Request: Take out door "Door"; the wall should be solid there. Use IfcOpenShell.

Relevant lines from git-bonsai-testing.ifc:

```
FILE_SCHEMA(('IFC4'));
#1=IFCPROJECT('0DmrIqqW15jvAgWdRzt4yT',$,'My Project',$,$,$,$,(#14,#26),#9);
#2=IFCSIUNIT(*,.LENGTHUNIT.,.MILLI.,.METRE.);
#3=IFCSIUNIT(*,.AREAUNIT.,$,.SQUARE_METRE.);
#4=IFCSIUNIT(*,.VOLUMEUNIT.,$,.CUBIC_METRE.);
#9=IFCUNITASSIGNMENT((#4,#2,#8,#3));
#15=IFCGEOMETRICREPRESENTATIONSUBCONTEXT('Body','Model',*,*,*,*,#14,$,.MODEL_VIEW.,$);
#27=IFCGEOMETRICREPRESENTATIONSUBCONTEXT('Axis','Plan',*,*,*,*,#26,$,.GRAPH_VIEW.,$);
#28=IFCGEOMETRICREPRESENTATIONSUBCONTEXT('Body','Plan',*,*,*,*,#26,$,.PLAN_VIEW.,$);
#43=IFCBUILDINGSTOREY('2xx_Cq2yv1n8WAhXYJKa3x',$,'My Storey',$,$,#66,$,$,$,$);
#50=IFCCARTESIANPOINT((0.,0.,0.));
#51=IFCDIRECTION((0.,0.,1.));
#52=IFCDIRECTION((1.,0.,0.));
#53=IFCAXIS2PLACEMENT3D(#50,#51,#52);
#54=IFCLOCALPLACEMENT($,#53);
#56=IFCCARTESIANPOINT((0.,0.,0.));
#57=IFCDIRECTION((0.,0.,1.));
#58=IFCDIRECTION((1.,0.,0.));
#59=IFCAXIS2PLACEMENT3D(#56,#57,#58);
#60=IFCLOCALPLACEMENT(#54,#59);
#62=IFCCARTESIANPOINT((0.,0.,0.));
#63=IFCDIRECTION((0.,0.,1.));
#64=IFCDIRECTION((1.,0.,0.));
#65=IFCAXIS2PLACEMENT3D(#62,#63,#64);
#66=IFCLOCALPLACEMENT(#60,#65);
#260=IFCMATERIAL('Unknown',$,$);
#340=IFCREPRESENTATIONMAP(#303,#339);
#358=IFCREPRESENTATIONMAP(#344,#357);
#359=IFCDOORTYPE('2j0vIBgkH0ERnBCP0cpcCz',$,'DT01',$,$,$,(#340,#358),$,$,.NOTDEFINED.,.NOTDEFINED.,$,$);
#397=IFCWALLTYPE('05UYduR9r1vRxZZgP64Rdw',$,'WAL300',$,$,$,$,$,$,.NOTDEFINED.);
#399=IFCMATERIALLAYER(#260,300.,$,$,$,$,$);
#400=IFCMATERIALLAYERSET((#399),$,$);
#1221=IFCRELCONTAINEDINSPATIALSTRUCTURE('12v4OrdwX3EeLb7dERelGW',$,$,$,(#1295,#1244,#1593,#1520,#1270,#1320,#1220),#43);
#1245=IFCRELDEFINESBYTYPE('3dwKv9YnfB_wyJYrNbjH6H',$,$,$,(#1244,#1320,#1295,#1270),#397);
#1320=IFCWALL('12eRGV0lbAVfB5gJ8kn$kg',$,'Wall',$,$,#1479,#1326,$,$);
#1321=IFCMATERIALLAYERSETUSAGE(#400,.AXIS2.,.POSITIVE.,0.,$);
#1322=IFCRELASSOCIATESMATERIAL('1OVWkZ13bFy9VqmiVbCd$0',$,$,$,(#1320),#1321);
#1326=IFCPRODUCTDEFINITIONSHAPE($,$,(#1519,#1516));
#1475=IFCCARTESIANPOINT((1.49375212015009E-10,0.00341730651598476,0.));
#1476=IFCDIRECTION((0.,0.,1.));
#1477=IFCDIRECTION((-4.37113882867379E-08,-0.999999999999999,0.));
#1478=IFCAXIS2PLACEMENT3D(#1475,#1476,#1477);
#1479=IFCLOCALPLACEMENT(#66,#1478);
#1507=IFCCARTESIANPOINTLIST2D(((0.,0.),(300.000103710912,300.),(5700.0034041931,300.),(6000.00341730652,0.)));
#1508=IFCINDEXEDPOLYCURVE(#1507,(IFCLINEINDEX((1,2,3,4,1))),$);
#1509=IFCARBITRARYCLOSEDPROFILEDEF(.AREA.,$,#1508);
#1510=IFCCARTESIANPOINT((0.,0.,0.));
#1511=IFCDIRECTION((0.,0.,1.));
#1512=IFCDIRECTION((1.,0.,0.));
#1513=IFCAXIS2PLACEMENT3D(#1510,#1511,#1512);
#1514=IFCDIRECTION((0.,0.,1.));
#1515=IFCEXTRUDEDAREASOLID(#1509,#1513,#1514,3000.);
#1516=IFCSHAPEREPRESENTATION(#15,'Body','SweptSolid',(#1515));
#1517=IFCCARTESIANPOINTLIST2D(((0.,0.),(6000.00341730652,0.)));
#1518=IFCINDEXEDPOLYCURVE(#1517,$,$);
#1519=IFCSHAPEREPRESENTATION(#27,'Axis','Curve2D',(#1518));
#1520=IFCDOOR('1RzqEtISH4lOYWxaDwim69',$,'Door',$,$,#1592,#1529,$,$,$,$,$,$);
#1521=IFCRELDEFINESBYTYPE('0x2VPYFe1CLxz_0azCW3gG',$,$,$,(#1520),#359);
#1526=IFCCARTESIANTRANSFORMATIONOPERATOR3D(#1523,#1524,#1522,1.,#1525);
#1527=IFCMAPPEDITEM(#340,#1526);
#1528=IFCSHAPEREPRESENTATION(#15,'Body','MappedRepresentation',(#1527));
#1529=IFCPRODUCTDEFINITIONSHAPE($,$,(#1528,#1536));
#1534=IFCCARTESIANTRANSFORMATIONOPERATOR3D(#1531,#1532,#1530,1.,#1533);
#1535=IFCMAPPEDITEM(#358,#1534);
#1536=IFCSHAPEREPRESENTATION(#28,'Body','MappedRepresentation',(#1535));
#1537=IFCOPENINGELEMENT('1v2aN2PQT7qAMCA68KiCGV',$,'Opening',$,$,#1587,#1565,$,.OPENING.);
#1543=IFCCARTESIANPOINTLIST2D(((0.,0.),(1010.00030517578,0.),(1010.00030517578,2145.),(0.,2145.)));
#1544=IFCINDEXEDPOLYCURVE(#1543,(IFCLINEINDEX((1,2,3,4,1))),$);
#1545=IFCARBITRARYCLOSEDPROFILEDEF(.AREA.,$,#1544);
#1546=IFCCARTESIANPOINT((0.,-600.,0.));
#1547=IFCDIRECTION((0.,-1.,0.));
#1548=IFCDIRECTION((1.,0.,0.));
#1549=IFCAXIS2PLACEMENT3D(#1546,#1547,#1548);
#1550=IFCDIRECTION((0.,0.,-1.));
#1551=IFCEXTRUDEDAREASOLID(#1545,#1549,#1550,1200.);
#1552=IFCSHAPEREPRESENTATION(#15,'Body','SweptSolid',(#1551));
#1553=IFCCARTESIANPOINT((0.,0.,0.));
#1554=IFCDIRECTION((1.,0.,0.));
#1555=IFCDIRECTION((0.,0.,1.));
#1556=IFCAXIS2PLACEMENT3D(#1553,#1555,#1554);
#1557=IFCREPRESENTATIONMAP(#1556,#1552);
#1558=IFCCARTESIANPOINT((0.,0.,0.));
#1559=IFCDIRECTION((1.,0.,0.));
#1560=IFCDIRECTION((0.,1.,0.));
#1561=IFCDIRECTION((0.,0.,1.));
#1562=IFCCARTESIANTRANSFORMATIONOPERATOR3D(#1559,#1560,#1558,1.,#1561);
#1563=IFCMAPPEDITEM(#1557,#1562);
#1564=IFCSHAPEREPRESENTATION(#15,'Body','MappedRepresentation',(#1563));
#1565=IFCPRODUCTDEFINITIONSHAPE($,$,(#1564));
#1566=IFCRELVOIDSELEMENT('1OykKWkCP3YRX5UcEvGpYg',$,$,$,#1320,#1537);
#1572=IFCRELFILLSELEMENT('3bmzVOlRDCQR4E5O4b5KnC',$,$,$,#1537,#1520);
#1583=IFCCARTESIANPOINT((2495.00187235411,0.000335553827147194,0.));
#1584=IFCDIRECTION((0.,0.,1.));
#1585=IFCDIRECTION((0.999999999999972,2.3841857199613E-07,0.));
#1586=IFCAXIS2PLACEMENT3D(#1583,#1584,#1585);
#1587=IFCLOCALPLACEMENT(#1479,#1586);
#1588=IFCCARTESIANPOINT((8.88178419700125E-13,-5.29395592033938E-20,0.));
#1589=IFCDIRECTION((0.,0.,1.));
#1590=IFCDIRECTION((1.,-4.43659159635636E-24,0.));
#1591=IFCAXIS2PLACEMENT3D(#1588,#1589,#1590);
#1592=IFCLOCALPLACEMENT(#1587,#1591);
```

```python
import ifcopenshell
import ifcopenshell.api.feature
import ifcopenshell.api.root
import ifcopenshell.geom
import ifcopenshell.util.shape

model = ifcopenshell.open("git-bonsai-testing.ifc")
settings = ifcopenshell.geom.settings()


def volume(element):
    """Net volume in cubic metres, openings subtracted."""
    shape = ifcopenshell.geom.create_shape(settings, element)
    return ifcopenshell.util.shape.get_volume(shape.geometry)


door = model.by_guid("1RzqEtISH4lOYWxaDwim69")
opening = door.FillsVoids[0].RelatingOpeningElement
wall = opening.VoidsElements[0].RelatingBuildingElement
before = volume(wall)

ifcopenshell.api.root.remove_product(model, product=door)
ifcopenshell.api.feature.remove_feature(model, feature=opening)

after = volume(wall)

print(f"wall volume {before:.3f} -> {after:.3f} m3")

model.write("git-bonsai-testing-out.ifc")
```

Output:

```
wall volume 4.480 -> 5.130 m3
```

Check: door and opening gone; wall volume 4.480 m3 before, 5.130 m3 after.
